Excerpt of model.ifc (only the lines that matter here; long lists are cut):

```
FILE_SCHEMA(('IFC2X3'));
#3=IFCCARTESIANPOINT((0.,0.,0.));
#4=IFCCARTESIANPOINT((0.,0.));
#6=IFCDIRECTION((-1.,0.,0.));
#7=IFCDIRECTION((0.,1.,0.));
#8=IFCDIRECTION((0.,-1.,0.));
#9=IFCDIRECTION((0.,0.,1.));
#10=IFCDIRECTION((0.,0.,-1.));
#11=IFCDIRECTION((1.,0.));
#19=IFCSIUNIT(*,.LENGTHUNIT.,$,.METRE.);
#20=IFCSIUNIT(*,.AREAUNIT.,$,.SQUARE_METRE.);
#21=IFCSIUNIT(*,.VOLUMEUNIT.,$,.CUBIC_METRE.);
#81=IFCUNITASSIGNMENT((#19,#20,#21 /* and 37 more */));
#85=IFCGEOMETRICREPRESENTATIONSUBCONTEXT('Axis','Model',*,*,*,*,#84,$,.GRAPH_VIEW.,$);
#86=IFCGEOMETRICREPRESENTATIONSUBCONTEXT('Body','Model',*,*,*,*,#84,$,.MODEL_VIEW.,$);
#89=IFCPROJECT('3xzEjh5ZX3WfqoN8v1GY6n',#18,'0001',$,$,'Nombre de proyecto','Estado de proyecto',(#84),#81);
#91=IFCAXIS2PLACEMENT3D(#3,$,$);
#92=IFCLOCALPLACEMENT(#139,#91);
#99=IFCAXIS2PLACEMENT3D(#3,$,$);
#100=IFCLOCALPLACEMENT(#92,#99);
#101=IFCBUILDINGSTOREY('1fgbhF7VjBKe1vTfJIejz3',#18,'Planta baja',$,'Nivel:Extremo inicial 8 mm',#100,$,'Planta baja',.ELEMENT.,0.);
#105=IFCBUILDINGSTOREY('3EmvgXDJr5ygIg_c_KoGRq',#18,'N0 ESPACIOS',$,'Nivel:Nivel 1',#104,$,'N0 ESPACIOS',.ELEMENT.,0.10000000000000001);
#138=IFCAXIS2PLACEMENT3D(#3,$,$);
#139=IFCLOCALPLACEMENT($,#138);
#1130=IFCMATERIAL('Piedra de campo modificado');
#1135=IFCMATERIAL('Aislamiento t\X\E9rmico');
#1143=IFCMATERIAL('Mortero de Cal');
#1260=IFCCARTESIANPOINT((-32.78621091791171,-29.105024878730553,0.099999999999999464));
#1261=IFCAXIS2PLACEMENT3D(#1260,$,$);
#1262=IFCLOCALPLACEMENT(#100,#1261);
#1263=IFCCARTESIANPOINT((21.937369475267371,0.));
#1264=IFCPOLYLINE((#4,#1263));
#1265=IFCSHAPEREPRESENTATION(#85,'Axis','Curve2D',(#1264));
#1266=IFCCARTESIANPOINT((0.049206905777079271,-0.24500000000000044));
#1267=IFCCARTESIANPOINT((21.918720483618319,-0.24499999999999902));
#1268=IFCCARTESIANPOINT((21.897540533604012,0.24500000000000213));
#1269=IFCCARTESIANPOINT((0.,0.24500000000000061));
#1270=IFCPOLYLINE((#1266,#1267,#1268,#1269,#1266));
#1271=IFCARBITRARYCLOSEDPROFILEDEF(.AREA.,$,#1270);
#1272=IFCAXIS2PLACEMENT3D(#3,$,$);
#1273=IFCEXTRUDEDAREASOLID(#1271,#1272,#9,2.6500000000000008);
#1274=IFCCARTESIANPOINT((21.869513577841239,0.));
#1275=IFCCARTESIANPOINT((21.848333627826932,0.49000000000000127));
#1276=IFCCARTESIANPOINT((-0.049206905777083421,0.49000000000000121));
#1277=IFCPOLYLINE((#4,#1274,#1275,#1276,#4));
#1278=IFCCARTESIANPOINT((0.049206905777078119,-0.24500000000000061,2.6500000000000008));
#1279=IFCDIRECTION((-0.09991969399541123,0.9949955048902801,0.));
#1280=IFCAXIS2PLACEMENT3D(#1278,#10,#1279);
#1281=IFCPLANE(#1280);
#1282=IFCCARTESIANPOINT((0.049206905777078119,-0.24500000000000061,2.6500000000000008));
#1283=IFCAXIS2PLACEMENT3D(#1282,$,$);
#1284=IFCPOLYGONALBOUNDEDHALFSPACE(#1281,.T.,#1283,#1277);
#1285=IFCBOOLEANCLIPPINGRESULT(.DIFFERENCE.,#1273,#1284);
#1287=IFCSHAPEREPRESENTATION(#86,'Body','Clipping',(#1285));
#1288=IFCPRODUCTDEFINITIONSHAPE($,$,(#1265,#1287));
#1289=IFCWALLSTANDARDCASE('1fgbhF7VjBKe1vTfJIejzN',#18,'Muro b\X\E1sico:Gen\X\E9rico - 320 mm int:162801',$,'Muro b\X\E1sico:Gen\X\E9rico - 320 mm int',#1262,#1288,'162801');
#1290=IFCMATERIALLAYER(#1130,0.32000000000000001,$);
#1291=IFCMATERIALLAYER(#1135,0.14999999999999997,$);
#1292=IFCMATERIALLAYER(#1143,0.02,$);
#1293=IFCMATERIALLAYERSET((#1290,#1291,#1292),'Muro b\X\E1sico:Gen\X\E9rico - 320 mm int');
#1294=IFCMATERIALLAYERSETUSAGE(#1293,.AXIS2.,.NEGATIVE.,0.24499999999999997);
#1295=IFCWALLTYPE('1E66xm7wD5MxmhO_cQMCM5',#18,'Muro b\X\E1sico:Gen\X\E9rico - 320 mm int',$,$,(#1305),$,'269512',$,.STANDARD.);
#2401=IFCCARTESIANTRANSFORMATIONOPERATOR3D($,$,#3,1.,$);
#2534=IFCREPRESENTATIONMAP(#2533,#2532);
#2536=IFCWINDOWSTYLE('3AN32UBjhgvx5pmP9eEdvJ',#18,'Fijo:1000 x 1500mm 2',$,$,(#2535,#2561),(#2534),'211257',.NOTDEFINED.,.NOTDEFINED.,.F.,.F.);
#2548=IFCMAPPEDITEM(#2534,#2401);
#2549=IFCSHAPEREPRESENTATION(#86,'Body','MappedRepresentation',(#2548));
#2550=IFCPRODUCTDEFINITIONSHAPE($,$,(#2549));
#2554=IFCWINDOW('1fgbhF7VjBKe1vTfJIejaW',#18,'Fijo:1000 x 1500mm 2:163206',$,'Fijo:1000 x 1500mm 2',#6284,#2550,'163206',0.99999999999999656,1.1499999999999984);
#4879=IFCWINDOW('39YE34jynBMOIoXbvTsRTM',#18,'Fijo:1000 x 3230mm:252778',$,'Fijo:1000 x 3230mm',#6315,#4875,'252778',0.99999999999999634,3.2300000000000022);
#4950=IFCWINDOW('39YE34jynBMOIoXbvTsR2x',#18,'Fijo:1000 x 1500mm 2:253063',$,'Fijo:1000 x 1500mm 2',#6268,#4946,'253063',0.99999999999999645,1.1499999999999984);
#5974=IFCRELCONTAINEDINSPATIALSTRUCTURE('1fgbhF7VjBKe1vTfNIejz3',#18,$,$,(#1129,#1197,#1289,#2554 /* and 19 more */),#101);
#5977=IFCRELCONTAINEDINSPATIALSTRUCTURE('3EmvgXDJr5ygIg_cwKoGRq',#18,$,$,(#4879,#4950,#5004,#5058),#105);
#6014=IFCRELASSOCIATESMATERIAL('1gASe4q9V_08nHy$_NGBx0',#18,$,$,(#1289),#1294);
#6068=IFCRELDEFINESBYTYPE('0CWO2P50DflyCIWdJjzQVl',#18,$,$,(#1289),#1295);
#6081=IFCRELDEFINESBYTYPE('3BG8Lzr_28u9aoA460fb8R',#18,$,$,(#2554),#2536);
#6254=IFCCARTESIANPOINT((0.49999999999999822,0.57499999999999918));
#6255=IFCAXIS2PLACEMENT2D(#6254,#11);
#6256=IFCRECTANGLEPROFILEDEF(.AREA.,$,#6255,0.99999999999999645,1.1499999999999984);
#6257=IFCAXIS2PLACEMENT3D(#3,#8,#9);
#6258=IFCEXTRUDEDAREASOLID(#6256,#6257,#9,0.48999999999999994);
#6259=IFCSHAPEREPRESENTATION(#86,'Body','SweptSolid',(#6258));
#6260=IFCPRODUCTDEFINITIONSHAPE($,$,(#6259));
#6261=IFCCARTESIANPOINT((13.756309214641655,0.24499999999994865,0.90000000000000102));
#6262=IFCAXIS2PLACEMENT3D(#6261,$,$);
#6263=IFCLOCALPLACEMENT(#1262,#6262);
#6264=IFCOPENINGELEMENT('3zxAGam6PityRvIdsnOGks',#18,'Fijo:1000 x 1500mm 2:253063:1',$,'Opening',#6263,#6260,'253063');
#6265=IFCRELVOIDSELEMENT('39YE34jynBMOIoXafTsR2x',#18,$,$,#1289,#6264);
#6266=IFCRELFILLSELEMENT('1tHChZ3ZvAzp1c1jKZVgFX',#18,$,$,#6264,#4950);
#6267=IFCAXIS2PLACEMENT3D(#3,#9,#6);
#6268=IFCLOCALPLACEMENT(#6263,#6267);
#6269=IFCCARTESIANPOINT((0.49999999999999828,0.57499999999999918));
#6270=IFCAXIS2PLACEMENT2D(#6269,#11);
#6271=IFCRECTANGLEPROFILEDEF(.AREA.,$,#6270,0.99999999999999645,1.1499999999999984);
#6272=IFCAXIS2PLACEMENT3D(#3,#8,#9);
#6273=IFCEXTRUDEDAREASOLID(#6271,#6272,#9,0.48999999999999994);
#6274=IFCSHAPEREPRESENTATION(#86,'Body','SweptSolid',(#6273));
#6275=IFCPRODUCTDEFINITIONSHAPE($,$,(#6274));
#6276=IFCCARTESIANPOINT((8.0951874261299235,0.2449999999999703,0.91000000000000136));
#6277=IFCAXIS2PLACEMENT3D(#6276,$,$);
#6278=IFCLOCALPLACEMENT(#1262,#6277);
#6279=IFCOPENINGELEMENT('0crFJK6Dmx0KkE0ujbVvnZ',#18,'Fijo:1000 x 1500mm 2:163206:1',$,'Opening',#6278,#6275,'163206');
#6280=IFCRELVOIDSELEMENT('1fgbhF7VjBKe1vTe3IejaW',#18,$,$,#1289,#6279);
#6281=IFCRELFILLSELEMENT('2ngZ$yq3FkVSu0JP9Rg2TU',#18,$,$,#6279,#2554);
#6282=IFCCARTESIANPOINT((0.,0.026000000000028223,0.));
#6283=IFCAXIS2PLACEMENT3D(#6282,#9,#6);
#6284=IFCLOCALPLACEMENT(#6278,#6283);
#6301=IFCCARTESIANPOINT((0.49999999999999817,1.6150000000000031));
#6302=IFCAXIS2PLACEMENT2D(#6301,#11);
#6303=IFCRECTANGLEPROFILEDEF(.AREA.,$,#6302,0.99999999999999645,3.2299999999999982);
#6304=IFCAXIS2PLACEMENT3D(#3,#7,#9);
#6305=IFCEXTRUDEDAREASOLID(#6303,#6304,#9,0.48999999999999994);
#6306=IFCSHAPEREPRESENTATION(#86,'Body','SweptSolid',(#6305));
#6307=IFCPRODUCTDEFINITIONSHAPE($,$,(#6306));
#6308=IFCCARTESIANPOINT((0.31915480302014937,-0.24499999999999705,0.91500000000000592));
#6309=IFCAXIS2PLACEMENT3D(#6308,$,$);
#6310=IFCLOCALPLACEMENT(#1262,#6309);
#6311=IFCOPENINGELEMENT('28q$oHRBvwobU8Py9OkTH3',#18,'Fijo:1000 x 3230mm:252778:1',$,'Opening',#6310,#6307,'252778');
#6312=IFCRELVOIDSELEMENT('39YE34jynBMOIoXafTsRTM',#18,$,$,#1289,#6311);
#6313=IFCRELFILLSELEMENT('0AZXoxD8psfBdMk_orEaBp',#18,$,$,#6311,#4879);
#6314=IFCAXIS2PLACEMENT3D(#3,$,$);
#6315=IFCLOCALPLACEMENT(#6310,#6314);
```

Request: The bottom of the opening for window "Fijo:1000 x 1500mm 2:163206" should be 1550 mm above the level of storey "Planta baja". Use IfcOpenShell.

```python
import numpy as np
import ifcopenshell
import ifcopenshell.api.geometry
import ifcopenshell.geom
import ifcopenshell.util.element
import ifcopenshell.util.placement
import ifcopenshell.util.shape
import ifcopenshell.util.unit

model = ifcopenshell.open("model.ifc")
unit_scale = ifcopenshell.util.unit.calculate_unit_scale(model)

window = model.by_guid("1fgbhF7VjBKe1vTfJIejaW")
opening = window.FillsVoids[0].RelatingOpeningElement
storey = ifcopenshell.util.element.get_container(window, ifc_class="IfcBuildingStorey")
level = ifcopenshell.util.placement.get_local_placement(storey.ObjectPlacement)[2, 3]

# The opening's origin need not be at the sill, so measure its lowest point.
shape = ifcopenshell.geom.create_shape(ifcopenshell.geom.settings(), opening)
bottom = ifcopenshell.util.shape.get_shape_bottom_elevation(shape, shape.geometry) / unit_scale
dz = level + 1.55 - bottom

shift = np.array([0.0, 0.0, dz])
# The window is placed relative to its opening, so it follows when the opening moves.
matrix = ifcopenshell.util.placement.get_local_placement(opening.ObjectPlacement)
matrix[:3, 3] += shift
ifcopenshell.api.geometry.edit_object_placement(
    model, product=opening, matrix=matrix, is_si=False, should_transform_children=True
)

print(f"moved by {dz * unit_scale:+.3f} m")

model.write("model_v2.ifc")
```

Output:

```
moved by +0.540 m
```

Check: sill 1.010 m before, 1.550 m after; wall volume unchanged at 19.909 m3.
